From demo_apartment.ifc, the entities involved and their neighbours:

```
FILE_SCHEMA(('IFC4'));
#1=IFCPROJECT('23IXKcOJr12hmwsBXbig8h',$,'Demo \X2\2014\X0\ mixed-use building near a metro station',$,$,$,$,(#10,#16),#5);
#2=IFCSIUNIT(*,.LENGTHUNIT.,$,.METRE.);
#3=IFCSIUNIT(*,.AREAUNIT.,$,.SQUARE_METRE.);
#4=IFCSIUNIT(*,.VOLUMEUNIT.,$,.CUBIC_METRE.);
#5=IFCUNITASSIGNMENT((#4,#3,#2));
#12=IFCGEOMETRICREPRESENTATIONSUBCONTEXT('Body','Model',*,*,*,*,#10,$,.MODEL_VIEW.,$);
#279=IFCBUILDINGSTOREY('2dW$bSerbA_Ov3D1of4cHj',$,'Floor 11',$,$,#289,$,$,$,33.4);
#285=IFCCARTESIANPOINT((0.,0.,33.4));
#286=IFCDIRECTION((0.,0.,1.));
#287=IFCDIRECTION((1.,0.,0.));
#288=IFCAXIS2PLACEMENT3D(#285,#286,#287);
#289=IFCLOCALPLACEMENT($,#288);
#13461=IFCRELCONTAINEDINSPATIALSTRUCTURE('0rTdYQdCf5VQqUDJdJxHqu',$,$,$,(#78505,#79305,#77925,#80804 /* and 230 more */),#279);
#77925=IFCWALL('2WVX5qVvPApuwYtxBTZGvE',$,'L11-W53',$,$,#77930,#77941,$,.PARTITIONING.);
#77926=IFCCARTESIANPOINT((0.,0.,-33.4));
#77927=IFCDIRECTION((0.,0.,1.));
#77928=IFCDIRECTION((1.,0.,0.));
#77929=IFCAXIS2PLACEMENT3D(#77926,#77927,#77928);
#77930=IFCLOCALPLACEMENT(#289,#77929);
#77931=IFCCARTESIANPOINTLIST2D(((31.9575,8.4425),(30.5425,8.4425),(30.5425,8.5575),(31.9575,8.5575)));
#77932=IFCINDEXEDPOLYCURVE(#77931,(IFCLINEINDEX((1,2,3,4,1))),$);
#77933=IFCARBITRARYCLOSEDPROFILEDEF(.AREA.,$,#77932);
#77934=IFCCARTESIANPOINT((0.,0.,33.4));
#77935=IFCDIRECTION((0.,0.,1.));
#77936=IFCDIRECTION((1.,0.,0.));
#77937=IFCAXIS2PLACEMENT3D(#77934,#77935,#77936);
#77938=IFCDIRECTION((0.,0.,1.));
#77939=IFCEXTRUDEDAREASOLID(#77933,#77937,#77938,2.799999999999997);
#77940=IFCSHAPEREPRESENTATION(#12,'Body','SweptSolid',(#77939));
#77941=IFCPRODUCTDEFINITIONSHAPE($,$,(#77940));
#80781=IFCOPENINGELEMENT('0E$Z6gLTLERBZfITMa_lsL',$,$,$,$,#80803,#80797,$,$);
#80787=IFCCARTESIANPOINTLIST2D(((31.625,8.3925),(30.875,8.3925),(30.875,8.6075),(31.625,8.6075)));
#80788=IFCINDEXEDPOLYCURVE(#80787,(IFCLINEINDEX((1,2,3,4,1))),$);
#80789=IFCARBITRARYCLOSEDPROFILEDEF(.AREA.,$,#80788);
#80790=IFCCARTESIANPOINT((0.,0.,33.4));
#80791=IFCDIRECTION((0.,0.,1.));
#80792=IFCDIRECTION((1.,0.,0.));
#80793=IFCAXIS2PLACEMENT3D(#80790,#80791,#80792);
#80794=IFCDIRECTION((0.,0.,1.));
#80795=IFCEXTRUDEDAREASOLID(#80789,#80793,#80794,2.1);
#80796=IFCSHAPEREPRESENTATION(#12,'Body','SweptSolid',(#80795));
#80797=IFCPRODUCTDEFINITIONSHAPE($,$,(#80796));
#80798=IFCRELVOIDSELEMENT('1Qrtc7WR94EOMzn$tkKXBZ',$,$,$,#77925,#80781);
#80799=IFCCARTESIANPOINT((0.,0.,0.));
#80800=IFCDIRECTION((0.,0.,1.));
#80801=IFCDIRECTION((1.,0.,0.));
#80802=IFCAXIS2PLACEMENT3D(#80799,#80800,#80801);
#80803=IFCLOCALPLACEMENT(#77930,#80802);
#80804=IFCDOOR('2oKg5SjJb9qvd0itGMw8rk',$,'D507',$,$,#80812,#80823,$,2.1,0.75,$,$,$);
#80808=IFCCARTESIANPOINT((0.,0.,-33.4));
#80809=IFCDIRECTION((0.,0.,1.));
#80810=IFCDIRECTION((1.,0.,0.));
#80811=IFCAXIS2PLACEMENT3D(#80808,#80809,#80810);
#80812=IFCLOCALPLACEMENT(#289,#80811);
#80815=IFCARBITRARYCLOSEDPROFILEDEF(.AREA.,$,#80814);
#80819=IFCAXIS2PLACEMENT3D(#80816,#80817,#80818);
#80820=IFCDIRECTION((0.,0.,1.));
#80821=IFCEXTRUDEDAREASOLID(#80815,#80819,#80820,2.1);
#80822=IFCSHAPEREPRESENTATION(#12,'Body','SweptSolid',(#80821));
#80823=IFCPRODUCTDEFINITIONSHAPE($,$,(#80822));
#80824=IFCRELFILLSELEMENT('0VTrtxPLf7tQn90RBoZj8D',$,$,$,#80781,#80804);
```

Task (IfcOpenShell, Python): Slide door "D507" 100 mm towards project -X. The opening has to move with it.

```python
import ifcopenshell
import ifcopenshell.api.geometry
import ifcopenshell.util.placement

model = ifcopenshell.open("demo_apartment.ifc")

door = model.by_guid("2oKg5SjJb9qvd0itGMw8rk")
opening = door.FillsVoids[0].RelatingOpeningElement
wall = opening.VoidsElements[0].RelatingBuildingElement

wall_matrix = ifcopenshell.util.placement.get_local_placement(wall.ObjectPlacement)
shift = wall_matrix[:3, 0] * -0.1
before = ifcopenshell.util.placement.get_local_placement(door.ObjectPlacement)[:3, 3].copy()

# The door is not placed relative to its opening, so move both.
for product in (opening, door):
    matrix = ifcopenshell.util.placement.get_local_placement(product.ObjectPlacement)
    matrix[:3, 3] += shift
    ifcopenshell.api.geometry.edit_object_placement(model, product=product, matrix=matrix, is_si=False)

after = ifcopenshell.util.placement.get_local_placement(door.ObjectPlacement)[:3, 3]
print("door moved by", (after - before).round(3) + 0.0)

model.write("demo_apartment_v2.ifc")
```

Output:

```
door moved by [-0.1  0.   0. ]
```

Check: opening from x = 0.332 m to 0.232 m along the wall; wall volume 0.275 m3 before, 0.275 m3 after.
